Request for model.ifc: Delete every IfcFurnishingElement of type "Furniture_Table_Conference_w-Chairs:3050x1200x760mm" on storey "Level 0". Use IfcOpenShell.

First a look at what the model holds.

```python
import ifcopenshell
import ifcopenshell.util.element

model = ifcopenshell.open("model.ifc")
print(model.schema)
storey = next(s for s in model.by_type("IfcBuildingStorey") if s.Name == "Level 0")
furniture = [e for e in ifcopenshell.util.element.get_decomposition(storey) if e.is_a("IfcFurnishingElement")]
seen = {}
for e in furniture:
    element_type = ifcopenshell.util.element.get_type(e)
    name = element_type.Name if element_type not in (None, e) else None
    seen[name] = seen.get(name, 0) + 1
for name, count in sorted(seen.items(), key=str):
    print(count, "x", name)
```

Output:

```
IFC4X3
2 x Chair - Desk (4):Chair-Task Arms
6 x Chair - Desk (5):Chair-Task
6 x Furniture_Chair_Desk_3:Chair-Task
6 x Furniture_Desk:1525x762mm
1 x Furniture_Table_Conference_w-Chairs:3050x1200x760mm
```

```python
import ifcopenshell
import ifcopenshell.api.root
import ifcopenshell.util.element

model = ifcopenshell.open("model.ifc")

storey = next(s for s in model.by_type("IfcBuildingStorey") if s.Name == "Level 0")
furniture = [e for e in ifcopenshell.util.element.get_decomposition(storey) if e.is_a("IfcFurnishingElement")]
targets = [e for e in furniture if (t := ifcopenshell.util.element.get_type(e)) not in (None, e) and t.Name == "Furniture_Table_Conference_w-Chairs:3050x1200x760mm"]

for e in targets:
    ifcopenshell.api.root.remove_product(model, product=e)
print(len(targets), "removed")

model.write("model_edited.ifc")
```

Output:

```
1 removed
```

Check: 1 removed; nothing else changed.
